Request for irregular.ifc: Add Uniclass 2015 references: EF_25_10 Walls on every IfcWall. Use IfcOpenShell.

First a look at what the model holds.

```python
import ifcopenshell

model = ifcopenshell.open("irregular.ifc")
print(model.schema)
print("classifications:", [c.Name for c in model.by_type("IfcClassification")])
for ifc_class in ("IfcDoor", "IfcRoof", "IfcStair", "IfcWall", "IfcWindow"):
    print(ifc_class, len(model.by_type(ifc_class)))
```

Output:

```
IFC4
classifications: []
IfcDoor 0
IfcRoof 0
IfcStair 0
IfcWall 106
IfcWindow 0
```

```python
import ifcopenshell
import ifcopenshell.api.classification

model = ifcopenshell.open("irregular.ifc")

system = ifcopenshell.api.classification.add_classification(model, classification="Uniclass 2015")

codes = {
    "IfcWall": ("EF_25_10", "Walls"),
}
for ifc_class, (code, name) in codes.items():
    products = model.by_type(ifc_class)
    ifcopenshell.api.classification.add_reference(
        model, products=products, classification=system, identification=code, name=name
    )
    print(code, len(products))

model.write("irregular_updated.ifc")
```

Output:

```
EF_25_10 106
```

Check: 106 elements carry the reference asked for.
